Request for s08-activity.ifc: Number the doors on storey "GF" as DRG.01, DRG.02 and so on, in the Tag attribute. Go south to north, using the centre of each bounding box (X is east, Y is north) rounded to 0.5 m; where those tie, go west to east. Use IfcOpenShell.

First a look at what the model holds.

```python
import ifcopenshell
import ifcopenshell.util.element
import ifcopenshell.util.placement

model = ifcopenshell.open("s08-activity.ifc")
print(model.schema)
storey = next(s for s in model.by_type("IfcBuildingStorey") if s.Name == "GF")
doors = [e for e in ifcopenshell.util.element.get_decomposition(storey) if e.is_a("IfcDoor")]
for e in sorted(doors, key=lambda e: e.id()):
    origin = ifcopenshell.util.placement.get_local_placement(e.ObjectPlacement)[:3, 3]
    print(e.id(), e.Tag, e.Name, origin.round(2) + 0.0, sep=" | ")
```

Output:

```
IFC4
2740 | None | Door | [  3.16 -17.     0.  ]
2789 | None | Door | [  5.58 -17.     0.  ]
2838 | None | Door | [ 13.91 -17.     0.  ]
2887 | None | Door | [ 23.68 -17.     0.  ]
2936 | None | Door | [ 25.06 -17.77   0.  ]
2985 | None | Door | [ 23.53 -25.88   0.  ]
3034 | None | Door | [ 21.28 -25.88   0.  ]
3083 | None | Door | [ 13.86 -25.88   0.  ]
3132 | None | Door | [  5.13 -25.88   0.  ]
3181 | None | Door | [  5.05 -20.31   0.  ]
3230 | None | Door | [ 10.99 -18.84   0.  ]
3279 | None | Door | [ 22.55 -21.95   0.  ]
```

```python
import ifcopenshell
import ifcopenshell.geom
import ifcopenshell.util.element
import ifcopenshell.util.shape

model = ifcopenshell.open("s08-activity.ifc")
settings = ifcopenshell.geom.settings()
settings.set("use-world-coords", True)


def centre(element):
    shape = ifcopenshell.geom.create_shape(settings, element)
    return ifcopenshell.util.shape.get_bbox_centroid(shape.geometry)


storey = next(s for s in model.by_type("IfcBuildingStorey") if s.Name == "GF")
doors = [e for e in ifcopenshell.util.element.get_decomposition(storey) if e.is_a("IfcDoor")]

# Insertion points can sit at a corner or the storey origin, so sort by the geometry (in metres).
centres = {e: centre(e) for e in doors}
doors.sort(key=lambda e: (round(centres[e][1] / 0.5), centres[e][0]))

for i, e in enumerate(doors, start=1):
    number = f"DRG.{i:02d}"
    e.Tag = number
    print(e.id(), number)

model.write("s08-activity_rev.ifc")
```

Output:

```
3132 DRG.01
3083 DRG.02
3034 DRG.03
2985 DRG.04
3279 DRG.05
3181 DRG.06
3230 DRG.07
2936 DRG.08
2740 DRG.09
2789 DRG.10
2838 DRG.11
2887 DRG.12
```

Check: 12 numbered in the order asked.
